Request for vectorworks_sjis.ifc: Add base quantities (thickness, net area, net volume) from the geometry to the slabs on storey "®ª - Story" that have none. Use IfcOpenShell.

First a look at what the model holds.

```python
import ifcopenshell
import ifcopenshell.util.element
import ifcopenshell.util.unit

model = ifcopenshell.open("vectorworks_sjis.ifc")
print(model.schema)
for unit_type in ("LENGTHUNIT", "AREAUNIT", "VOLUMEUNIT"):
    print(unit_type, ifcopenshell.util.unit.calculate_unit_scale(model, unit_type))
storey = next(s for s in model.by_type("IfcBuildingStorey") if s.Name == '\x89®\x8dª - Story')
slabs = [e for e in ifcopenshell.util.element.get_decomposition(storey) if e.is_a("IfcSlab")]
for e in sorted(slabs, key=lambda e: e.id()):
    print(e.id(), e.is_a(), e.Name, list(ifcopenshell.util.element.get_psets(e, qtos_only=True)), sep=" | ")
```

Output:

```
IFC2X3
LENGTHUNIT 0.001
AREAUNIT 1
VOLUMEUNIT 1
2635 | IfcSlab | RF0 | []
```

```python
import ifcopenshell
import ifcopenshell.api.pset
import ifcopenshell.geom
import ifcopenshell.util.element
import ifcopenshell.util.shape
import ifcopenshell.util.unit

model = ifcopenshell.open("vectorworks_sjis.ifc")
unit_scale = ifcopenshell.util.unit.calculate_unit_scale(model)
area_scale = ifcopenshell.util.unit.calculate_unit_scale(model, "AREAUNIT")
volume_scale = ifcopenshell.util.unit.calculate_unit_scale(model, "VOLUMEUNIT")
settings = ifcopenshell.geom.settings()

storey = next(s for s in model.by_type("IfcBuildingStorey") if s.Name == '\x89®\x8dª - Story')
slabs = [e for e in ifcopenshell.util.element.get_decomposition(storey) if e.is_a("IfcSlab")]

for e in sorted(slabs, key=lambda e: e.id()):
    if ifcopenshell.util.element.get_psets(e, qtos_only=True, should_inherit=False):
        continue
    # Geometry comes back in metres, in the element's own axes.
    shape = ifcopenshell.geom.create_shape(settings, e)
    values = {
        "Width": ifcopenshell.util.shape.get_z(shape.geometry) / unit_scale,
        "NetArea": ifcopenshell.util.shape.get_footprint_area(shape.geometry) / area_scale,
        "NetVolume": ifcopenshell.util.shape.get_volume(shape.geometry) / volume_scale,
    }
    qto = ifcopenshell.api.pset.add_qto(model, product=e, name="BaseQuantities")
    ifcopenshell.api.pset.edit_qto(model, qto=qto, properties=values)
    print(e.id(), {k: round(v, 3) for k, v in values.items()})

model.write("vectorworks_sjis_v2.ifc")
```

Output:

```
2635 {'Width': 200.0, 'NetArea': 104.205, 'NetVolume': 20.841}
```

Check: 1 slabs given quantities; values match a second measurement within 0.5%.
